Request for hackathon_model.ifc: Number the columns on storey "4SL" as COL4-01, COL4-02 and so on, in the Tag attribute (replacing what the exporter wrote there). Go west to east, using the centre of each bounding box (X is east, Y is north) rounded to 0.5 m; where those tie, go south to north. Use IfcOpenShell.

First a look at what the model holds.

```python
import ifcopenshell
import ifcopenshell.util.element
import ifcopenshell.util.placement

model = ifcopenshell.open("hackathon_model.ifc")
print(model.schema)
storey = next(s for s in model.by_type("IfcBuildingStorey") if s.Name == "4SL")
columns = [e for e in ifcopenshell.util.element.get_decomposition(storey) if e.is_a("IfcColumn")]
for e in sorted(columns, key=lambda e: e.id()):
    origin = ifcopenshell.util.placement.get_local_placement(e.ObjectPlacement)[:3, 3]
    print(e.id(), e.Tag, e.Name, origin.round(2) + 0.0, sep=" | ")
```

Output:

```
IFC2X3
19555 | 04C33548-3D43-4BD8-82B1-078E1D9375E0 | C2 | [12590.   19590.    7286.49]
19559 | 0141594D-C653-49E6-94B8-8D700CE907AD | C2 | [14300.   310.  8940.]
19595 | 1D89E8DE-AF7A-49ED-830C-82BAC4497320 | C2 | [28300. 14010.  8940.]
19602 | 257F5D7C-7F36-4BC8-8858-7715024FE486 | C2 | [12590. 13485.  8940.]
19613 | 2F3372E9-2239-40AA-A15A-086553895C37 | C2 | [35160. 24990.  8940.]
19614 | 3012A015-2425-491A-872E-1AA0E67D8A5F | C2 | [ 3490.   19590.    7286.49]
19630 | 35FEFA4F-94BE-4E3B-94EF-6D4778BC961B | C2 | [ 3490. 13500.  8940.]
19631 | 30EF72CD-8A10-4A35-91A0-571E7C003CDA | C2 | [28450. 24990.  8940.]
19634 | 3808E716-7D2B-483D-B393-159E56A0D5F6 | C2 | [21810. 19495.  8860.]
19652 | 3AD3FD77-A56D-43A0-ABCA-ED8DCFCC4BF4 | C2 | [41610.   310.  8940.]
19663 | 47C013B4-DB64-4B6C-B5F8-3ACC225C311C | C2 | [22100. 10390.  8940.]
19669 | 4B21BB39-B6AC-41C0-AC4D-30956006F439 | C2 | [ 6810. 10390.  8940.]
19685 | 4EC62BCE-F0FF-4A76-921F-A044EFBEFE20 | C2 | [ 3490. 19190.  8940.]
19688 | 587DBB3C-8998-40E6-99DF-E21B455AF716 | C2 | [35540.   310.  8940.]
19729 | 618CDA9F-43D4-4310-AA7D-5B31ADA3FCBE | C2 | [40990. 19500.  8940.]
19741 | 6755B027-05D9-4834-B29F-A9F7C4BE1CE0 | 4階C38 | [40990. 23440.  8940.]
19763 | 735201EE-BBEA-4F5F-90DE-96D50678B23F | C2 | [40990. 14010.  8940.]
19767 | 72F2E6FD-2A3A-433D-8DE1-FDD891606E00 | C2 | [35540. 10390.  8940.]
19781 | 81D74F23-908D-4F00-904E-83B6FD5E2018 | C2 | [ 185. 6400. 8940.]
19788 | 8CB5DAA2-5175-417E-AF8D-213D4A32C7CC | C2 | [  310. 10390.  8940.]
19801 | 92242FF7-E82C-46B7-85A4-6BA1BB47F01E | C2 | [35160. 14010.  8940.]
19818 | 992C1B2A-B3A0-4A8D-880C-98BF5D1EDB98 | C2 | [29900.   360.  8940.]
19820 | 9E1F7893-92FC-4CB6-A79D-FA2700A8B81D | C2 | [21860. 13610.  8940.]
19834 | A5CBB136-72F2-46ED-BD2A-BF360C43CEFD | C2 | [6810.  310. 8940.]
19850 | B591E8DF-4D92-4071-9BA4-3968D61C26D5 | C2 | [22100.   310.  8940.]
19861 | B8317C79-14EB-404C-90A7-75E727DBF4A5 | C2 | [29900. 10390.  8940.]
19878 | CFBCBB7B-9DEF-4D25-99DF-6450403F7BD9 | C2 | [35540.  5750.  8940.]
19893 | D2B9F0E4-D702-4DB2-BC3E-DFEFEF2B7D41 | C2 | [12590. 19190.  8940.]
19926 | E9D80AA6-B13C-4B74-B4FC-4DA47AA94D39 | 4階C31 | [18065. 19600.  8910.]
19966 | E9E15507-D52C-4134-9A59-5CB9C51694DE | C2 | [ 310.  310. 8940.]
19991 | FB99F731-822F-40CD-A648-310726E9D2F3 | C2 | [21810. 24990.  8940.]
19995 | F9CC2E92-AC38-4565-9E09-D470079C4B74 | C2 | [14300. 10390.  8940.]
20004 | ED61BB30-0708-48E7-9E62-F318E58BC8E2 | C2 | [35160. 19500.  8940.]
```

```python
import ifcopenshell
import ifcopenshell.geom
import ifcopenshell.util.element
import ifcopenshell.util.shape

model = ifcopenshell.open("hackathon_model.ifc")
settings = ifcopenshell.geom.settings()
settings.set("use-world-coords", True)


def centre(element):
    shape = ifcopenshell.geom.create_shape(settings, element)
    return ifcopenshell.util.shape.get_bbox_centroid(shape.geometry)


storey = next(s for s in model.by_type("IfcBuildingStorey") if s.Name == "4SL")
columns = [e for e in ifcopenshell.util.element.get_decomposition(storey) if e.is_a("IfcColumn")]

# Insertion points can sit at a corner or the storey origin, so sort by the geometry (in metres).
centres = {e: centre(e) for e in columns}
columns.sort(key=lambda e: (round(centres[e][0] / 0.5), centres[e][1]))

for i, e in enumerate(columns, start=1):
    number = f"COL4-{i:02d}"
    e.Tag = number
    print(e.id(), number)

model.write("hackathon_model_v2.ifc")
```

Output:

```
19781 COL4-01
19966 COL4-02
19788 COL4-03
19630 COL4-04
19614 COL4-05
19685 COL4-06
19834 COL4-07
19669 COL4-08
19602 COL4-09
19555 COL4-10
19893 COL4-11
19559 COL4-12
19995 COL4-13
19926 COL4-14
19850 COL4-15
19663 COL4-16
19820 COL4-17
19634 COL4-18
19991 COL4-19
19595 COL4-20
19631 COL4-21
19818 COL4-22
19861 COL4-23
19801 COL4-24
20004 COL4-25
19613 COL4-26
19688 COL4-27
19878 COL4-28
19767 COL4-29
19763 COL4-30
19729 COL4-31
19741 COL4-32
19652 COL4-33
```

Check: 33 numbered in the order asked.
